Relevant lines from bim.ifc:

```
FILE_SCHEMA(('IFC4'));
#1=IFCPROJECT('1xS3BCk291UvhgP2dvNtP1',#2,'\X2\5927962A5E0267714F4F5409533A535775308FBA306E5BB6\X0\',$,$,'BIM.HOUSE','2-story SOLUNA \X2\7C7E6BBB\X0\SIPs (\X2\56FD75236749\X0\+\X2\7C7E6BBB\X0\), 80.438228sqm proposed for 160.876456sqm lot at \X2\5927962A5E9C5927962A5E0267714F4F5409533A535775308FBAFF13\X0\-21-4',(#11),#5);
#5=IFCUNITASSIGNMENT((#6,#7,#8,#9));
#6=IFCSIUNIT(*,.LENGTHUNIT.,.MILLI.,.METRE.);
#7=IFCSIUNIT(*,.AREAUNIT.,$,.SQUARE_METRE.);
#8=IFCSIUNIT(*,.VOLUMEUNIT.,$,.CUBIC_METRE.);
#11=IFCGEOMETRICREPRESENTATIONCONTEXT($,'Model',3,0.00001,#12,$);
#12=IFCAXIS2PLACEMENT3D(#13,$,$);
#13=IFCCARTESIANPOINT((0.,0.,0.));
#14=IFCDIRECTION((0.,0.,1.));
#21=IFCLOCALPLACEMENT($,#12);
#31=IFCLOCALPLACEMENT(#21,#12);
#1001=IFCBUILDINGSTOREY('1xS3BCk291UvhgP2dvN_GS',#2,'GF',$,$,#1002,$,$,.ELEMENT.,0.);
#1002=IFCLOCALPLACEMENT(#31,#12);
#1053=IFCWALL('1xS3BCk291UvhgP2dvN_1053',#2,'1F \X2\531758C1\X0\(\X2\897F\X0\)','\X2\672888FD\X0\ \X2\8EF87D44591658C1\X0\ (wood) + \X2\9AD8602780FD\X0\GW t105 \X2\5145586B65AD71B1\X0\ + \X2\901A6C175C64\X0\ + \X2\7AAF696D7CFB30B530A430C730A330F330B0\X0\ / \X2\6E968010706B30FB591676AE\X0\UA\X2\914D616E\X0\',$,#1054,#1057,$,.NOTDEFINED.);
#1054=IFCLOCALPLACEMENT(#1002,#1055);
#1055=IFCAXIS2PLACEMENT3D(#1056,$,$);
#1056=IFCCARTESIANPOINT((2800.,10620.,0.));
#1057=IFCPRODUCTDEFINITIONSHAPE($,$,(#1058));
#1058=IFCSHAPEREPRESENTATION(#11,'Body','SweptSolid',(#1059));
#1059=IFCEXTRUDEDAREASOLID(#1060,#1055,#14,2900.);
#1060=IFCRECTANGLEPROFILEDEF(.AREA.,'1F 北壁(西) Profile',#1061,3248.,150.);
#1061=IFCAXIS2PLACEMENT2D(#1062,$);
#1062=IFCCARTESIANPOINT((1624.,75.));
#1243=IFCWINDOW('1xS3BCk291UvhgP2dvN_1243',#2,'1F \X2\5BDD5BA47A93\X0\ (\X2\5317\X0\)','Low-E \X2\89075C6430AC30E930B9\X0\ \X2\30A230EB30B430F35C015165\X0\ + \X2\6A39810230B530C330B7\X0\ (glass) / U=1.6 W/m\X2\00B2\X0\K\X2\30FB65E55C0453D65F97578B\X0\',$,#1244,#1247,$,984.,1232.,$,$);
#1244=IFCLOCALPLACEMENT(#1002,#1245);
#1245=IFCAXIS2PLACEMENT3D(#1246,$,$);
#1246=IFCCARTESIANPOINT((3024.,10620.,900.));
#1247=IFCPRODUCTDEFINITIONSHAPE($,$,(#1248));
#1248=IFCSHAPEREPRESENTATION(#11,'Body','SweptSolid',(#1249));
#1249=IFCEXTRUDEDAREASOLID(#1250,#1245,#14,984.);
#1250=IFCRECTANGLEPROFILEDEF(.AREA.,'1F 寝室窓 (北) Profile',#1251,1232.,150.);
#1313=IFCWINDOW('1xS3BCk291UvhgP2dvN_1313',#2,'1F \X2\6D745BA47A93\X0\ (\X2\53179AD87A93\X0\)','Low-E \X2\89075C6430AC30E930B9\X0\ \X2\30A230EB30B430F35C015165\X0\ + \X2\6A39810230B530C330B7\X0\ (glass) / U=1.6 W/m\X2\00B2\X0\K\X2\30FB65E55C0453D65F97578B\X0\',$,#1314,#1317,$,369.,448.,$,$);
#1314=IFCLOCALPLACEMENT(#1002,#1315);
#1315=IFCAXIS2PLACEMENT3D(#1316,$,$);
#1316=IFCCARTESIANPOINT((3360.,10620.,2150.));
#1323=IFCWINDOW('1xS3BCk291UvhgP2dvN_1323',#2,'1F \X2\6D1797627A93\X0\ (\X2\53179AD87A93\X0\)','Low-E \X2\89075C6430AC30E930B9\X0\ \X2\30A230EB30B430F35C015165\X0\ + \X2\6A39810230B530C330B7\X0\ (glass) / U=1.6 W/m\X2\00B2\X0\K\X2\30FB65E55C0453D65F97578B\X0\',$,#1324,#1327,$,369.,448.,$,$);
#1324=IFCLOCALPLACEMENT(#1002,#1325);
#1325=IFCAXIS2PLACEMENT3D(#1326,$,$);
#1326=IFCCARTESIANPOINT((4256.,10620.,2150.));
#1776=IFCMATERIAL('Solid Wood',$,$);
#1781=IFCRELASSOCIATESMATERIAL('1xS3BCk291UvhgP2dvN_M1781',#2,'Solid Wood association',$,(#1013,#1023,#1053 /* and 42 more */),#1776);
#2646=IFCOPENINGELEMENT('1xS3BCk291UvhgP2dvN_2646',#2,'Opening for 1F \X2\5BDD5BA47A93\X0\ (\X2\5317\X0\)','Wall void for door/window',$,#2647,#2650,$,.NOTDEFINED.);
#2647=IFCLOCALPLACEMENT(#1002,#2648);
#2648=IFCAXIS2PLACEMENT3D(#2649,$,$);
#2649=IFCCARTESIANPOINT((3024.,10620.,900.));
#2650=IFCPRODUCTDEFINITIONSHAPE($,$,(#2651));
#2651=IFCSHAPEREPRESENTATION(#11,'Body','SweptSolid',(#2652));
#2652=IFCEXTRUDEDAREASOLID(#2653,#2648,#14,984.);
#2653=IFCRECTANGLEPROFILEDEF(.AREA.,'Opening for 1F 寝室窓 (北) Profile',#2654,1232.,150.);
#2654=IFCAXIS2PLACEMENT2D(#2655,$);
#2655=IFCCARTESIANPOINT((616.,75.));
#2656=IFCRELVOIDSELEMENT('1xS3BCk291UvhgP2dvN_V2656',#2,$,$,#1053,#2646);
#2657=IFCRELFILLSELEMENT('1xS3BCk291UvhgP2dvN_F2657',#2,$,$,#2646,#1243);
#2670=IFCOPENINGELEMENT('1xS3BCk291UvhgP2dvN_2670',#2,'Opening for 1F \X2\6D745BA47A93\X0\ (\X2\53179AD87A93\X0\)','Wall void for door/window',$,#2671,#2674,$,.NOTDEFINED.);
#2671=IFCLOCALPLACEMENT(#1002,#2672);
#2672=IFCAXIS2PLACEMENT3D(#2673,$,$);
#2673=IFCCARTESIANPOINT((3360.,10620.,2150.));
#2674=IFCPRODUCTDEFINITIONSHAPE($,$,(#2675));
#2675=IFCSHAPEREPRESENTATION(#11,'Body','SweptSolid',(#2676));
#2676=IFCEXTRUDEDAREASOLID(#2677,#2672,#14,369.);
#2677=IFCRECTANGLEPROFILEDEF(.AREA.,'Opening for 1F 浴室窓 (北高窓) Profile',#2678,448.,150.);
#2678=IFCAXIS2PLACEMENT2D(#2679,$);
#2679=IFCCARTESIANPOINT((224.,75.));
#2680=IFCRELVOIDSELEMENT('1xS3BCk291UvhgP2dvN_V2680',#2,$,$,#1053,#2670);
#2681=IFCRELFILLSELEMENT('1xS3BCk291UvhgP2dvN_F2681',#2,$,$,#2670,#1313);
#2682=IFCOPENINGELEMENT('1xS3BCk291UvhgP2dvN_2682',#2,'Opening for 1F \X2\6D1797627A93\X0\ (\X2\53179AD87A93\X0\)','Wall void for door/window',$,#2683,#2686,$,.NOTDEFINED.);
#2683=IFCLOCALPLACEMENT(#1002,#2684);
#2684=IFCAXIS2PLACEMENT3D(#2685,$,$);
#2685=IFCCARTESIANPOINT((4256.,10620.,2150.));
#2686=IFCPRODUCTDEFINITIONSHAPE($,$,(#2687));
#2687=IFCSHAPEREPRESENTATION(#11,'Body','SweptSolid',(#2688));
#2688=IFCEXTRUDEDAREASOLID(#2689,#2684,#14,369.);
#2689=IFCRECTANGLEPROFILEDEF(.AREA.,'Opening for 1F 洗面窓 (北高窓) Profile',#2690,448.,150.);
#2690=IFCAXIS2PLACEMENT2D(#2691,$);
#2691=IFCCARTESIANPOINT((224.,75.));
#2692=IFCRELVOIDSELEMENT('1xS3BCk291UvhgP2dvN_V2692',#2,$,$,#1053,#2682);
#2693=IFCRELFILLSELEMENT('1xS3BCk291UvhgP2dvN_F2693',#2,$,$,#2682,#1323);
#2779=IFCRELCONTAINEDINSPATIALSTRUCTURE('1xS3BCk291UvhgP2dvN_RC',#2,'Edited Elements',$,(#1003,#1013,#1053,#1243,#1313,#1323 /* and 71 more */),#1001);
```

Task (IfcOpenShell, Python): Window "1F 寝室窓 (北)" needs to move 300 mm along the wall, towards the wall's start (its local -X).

```python
import ifcopenshell
import ifcopenshell.api.geometry
import ifcopenshell.util.placement
import ifcopenshell.util.unit

model = ifcopenshell.open("bim.ifc")
unit_scale = ifcopenshell.util.unit.calculate_unit_scale(model)

window = model.by_id(1243)
opening = window.FillsVoids[0].RelatingOpeningElement
wall = opening.VoidsElements[0].RelatingBuildingElement

wall_matrix = ifcopenshell.util.placement.get_local_placement(wall.ObjectPlacement)
shift = wall_matrix[:3, 0] * -0.3 / unit_scale
before = ifcopenshell.util.placement.get_local_placement(window.ObjectPlacement)[:3, 3].copy()

# The window is not placed relative to its opening, so move both.
for product in (opening, window):
    matrix = ifcopenshell.util.placement.get_local_placement(product.ObjectPlacement)
    matrix[:3, 3] += shift
    ifcopenshell.api.geometry.edit_object_placement(model, product=product, matrix=matrix, is_si=False)

after = ifcopenshell.util.placement.get_local_placement(window.ObjectPlacement)[:3, 3]
print("window moved by", (after - before).round(3) + 0.0)

model.write("bim_v2.ifc")
```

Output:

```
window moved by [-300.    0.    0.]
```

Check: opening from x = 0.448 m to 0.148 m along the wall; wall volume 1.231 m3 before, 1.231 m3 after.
